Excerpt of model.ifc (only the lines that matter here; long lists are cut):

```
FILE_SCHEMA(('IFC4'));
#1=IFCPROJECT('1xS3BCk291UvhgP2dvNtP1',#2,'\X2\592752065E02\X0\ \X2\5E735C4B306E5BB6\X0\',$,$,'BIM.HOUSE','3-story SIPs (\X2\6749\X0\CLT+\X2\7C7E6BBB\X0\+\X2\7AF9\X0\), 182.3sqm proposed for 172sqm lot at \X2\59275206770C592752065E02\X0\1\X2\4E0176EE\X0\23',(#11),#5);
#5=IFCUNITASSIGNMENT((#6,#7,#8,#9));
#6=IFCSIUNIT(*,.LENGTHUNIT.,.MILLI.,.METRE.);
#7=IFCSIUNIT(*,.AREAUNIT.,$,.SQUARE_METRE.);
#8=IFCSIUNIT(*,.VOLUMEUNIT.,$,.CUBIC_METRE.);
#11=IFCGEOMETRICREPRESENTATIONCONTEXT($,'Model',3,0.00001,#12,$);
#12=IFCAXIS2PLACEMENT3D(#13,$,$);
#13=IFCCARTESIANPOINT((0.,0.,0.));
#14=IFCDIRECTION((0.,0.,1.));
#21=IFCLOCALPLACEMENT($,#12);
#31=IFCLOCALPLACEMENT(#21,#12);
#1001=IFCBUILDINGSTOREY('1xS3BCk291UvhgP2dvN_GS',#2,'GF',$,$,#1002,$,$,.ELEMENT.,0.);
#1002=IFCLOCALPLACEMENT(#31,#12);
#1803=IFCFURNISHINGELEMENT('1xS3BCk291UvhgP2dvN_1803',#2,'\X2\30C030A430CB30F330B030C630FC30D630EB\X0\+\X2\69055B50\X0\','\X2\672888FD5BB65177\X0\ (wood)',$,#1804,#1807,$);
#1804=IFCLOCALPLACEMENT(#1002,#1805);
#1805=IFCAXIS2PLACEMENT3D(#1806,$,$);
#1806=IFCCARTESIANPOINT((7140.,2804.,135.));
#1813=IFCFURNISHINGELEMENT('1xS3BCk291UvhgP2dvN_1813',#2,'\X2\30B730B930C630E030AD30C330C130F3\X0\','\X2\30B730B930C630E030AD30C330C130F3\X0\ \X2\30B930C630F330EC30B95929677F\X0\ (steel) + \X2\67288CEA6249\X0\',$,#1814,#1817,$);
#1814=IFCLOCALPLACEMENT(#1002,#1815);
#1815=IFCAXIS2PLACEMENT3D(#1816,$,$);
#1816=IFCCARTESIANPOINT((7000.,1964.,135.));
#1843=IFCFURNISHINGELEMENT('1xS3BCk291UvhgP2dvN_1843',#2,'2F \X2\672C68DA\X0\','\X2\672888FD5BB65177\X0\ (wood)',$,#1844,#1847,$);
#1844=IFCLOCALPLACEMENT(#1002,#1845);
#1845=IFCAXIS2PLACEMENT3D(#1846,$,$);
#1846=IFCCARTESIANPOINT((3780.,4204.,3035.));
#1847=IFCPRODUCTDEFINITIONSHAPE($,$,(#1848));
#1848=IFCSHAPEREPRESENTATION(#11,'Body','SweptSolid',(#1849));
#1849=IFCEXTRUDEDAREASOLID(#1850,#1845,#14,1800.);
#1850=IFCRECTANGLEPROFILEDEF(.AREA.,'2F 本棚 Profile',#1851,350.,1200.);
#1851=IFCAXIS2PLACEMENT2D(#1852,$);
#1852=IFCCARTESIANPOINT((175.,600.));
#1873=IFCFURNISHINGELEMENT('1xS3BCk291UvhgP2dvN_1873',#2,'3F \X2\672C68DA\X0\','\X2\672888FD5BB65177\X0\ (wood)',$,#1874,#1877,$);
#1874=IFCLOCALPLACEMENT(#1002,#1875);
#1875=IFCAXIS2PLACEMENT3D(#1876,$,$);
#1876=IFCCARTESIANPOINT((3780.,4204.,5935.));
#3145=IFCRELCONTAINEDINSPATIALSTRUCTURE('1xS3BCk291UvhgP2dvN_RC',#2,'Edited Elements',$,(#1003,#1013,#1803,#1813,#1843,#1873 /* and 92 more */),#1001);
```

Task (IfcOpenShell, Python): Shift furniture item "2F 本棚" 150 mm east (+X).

```python
import ifcopenshell
import ifcopenshell.api.geometry
import ifcopenshell.util.placement
import ifcopenshell.util.unit

model = ifcopenshell.open("model.ifc")
unit_scale = ifcopenshell.util.unit.calculate_unit_scale(model)

item = model.by_id(1843)
matrix = ifcopenshell.util.placement.get_local_placement(item.ObjectPlacement)
matrix[0, 3] += 0.15 / unit_scale
ifcopenshell.api.geometry.edit_object_placement(model, product=item, matrix=matrix, is_si=False)

print(ifcopenshell.util.placement.get_local_placement(item.ObjectPlacement).round(3) + 0.0)

model.write("model_rev.ifc")
```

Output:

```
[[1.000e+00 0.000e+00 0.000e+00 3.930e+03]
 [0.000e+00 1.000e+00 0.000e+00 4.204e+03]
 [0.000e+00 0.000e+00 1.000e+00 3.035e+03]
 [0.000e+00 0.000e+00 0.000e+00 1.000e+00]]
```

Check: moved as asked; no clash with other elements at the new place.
